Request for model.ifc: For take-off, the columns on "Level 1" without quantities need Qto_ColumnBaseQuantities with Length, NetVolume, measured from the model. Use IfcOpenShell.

First a look at what the model holds.

```python
import ifcopenshell
import ifcopenshell.util.element
import ifcopenshell.util.unit

model = ifcopenshell.open("model.ifc")
print(model.schema)
for unit_type in ("LENGTHUNIT", "AREAUNIT", "VOLUMEUNIT"):
    print(unit_type, ifcopenshell.util.unit.calculate_unit_scale(model, unit_type))
storey = next(s for s in model.by_type("IfcBuildingStorey") if s.Name == "Level 1")
columns = [e for e in ifcopenshell.util.element.get_decomposition(storey) if e.is_a("IfcColumn")]
for e in sorted(columns, key=lambda e: e.id()):
    print(e.id(), e.is_a(), e.Name, list(ifcopenshell.util.element.get_psets(e, qtos_only=True)), sep=" | ")
```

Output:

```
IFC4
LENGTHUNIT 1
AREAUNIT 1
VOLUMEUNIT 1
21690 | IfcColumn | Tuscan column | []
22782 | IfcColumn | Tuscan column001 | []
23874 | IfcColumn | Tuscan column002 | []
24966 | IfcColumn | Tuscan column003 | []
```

```python
import ifcopenshell
import ifcopenshell.api.pset
import ifcopenshell.geom
import ifcopenshell.util.element
import ifcopenshell.util.shape
import ifcopenshell.util.unit

model = ifcopenshell.open("model.ifc")
unit_scale = ifcopenshell.util.unit.calculate_unit_scale(model)
volume_scale = ifcopenshell.util.unit.calculate_unit_scale(model, "VOLUMEUNIT")
settings = ifcopenshell.geom.settings()

storey = next(s for s in model.by_type("IfcBuildingStorey") if s.Name == "Level 1")
columns = [e for e in ifcopenshell.util.element.get_decomposition(storey) if e.is_a("IfcColumn")]

for e in sorted(columns, key=lambda e: e.id()):
    if ifcopenshell.util.element.get_psets(e, qtos_only=True, should_inherit=False):
        continue
    # Geometry comes back in metres, in the element's own axes.
    shape = ifcopenshell.geom.create_shape(settings, e)
    values = {
        "Length": ifcopenshell.util.shape.get_z(shape.geometry) / unit_scale,
        "NetVolume": ifcopenshell.util.shape.get_volume(shape.geometry) / volume_scale,
    }
    qto = ifcopenshell.api.pset.add_qto(model, product=e, name="Qto_ColumnBaseQuantities")
    ifcopenshell.api.pset.edit_qto(model, qto=qto, properties=values)
    print(e.id(), {k: round(v, 3) for k, v in values.items()})

model.write("model_edited.ifc")
```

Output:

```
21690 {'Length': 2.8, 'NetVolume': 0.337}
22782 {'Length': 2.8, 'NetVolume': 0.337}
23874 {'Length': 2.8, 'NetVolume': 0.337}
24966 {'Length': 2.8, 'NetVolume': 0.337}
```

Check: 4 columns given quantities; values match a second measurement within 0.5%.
